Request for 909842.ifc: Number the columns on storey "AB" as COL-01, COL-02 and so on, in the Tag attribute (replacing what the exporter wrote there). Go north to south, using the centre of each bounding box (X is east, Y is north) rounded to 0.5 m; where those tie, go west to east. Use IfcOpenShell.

First a look at what the model holds.

```python
import ifcopenshell
import ifcopenshell.util.element
import ifcopenshell.util.placement

model = ifcopenshell.open("909842.ifc")
print(model.schema)
storey = next(s for s in model.by_type("IfcBuildingStorey") if s.Name == "AB")
columns = [e for e in ifcopenshell.util.element.get_decomposition(storey) if e.is_a("IfcColumn")]
for e in sorted(columns, key=lambda e: e.id()):
    origin = ifcopenshell.util.placement.get_local_placement(e.ObjectPlacement)[:3, 3]
    print(e.id(), e.Tag, e.Name, origin.round(2) + 0.0, sep=" | ")
```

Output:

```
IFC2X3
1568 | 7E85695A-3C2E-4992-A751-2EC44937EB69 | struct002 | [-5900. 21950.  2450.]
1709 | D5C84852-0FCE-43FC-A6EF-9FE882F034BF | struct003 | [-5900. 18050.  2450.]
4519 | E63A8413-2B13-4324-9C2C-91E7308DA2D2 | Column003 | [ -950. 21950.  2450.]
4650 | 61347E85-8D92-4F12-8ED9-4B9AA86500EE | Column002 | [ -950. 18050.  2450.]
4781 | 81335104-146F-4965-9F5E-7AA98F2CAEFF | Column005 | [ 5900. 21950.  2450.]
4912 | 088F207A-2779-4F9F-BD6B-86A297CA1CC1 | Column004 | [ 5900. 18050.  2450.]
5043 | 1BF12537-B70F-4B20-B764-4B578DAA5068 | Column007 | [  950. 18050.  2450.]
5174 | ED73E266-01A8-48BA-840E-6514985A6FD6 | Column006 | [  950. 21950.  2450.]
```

```python
import ifcopenshell
import ifcopenshell.geom
import ifcopenshell.util.element
import ifcopenshell.util.shape

model = ifcopenshell.open("909842.ifc")
settings = ifcopenshell.geom.settings()
settings.set("use-world-coords", True)


def centre(element):
    shape = ifcopenshell.geom.create_shape(settings, element)
    return ifcopenshell.util.shape.get_bbox_centroid(shape.geometry)


storey = next(s for s in model.by_type("IfcBuildingStorey") if s.Name == "AB")
columns = [e for e in ifcopenshell.util.element.get_decomposition(storey) if e.is_a("IfcColumn")]

# Insertion points can sit at a corner or the storey origin, so sort by the geometry (in metres).
centres = {e: centre(e) for e in columns}
columns.sort(key=lambda e: (-round(centres[e][1] / 0.5), centres[e][0]))

for i, e in enumerate(columns, start=1):
    number = f"COL-{i:02d}"
    e.Tag = number
    print(e.id(), number)

model.write("909842_edited.ifc")
```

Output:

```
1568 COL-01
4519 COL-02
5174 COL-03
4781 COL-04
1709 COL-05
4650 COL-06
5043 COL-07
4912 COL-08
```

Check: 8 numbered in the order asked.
